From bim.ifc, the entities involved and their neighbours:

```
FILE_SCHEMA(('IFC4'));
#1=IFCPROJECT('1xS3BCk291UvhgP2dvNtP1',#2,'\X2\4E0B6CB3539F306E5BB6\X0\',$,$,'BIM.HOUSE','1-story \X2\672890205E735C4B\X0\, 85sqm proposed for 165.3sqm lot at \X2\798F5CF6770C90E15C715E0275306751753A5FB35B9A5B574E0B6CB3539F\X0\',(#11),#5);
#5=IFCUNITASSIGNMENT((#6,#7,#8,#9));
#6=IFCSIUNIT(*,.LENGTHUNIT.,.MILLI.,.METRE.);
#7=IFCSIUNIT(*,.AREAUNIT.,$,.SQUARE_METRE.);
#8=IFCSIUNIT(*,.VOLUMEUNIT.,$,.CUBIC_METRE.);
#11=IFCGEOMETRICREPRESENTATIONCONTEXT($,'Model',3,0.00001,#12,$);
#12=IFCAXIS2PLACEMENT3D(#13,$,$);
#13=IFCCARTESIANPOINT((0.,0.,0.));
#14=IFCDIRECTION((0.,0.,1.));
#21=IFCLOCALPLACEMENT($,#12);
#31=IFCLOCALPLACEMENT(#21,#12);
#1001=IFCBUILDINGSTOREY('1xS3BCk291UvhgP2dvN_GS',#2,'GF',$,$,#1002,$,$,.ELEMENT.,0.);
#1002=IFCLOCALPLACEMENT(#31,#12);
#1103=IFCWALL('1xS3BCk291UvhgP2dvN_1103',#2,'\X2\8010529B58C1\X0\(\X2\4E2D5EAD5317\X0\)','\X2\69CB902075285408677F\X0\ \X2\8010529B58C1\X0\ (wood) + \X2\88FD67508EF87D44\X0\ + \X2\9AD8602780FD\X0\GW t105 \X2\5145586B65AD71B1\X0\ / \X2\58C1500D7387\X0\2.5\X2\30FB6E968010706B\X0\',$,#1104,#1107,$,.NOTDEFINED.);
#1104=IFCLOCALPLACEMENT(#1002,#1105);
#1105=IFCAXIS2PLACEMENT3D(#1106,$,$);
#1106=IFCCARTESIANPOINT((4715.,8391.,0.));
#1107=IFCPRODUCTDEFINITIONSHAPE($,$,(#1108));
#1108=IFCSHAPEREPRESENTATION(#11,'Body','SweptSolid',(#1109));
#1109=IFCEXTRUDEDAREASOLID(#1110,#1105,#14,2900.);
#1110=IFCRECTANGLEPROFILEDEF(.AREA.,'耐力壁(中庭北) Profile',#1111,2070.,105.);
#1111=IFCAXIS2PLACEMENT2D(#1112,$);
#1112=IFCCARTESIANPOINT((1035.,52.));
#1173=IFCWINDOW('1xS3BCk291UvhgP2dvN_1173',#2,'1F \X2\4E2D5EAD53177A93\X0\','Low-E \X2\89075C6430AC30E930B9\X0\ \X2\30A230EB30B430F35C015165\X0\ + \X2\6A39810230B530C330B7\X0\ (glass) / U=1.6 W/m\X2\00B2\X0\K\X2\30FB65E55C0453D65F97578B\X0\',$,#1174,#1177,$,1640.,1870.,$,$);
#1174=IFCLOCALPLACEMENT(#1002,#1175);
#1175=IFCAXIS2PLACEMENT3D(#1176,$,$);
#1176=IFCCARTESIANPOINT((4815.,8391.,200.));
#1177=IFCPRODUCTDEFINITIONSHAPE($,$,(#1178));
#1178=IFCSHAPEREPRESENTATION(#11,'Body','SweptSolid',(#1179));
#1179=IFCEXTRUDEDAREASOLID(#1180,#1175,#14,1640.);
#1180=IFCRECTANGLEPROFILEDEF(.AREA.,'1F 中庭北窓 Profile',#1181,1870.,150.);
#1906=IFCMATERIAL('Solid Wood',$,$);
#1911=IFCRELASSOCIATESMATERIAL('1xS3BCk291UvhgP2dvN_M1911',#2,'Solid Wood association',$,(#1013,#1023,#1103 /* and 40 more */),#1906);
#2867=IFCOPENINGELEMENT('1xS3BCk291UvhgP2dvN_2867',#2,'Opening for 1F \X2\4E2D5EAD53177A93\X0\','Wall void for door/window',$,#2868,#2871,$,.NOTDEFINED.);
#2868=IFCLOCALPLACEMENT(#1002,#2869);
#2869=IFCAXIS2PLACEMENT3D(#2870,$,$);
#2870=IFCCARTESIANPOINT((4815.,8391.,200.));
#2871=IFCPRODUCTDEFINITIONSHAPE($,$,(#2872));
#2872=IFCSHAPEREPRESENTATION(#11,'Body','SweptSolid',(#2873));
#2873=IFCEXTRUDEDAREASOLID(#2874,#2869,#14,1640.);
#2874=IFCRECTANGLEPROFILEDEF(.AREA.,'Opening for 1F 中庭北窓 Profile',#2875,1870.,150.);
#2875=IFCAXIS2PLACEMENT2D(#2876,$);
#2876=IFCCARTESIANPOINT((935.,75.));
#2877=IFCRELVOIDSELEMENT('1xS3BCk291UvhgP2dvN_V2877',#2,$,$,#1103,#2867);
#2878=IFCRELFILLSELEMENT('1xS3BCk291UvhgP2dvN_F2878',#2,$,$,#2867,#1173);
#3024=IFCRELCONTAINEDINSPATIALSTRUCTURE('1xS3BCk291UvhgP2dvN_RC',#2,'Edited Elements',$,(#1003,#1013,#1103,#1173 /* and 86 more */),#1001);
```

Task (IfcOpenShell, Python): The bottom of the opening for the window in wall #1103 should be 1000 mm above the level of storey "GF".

```python
import numpy as np
import ifcopenshell
import ifcopenshell.api.geometry
import ifcopenshell.geom
import ifcopenshell.util.element
import ifcopenshell.util.placement
import ifcopenshell.util.shape
import ifcopenshell.util.unit

model = ifcopenshell.open("bim.ifc")
unit_scale = ifcopenshell.util.unit.calculate_unit_scale(model)

window = model.by_guid("1xS3BCk291UvhgP2dvN_1173")
opening = window.FillsVoids[0].RelatingOpeningElement
storey = ifcopenshell.util.element.get_container(window, ifc_class="IfcBuildingStorey")
level = ifcopenshell.util.placement.get_local_placement(storey.ObjectPlacement)[2, 3]

# The opening's origin need not be at the sill, so measure its lowest point.
shape = ifcopenshell.geom.create_shape(ifcopenshell.geom.settings(), opening)
bottom = ifcopenshell.util.shape.get_shape_bottom_elevation(shape, shape.geometry) / unit_scale
dz = level + 1000.0 - bottom

shift = np.array([0.0, 0.0, dz])
# The window is not placed relative to its opening, so move both.
for product in (opening, window):
    matrix = ifcopenshell.util.placement.get_local_placement(product.ObjectPlacement)
    matrix[:3, 3] += shift
    ifcopenshell.api.geometry.edit_object_placement(model, product=product, matrix=matrix, is_si=False)

print(f"moved by {dz * unit_scale:+.3f} m")

model.write("bim-out.ifc")
```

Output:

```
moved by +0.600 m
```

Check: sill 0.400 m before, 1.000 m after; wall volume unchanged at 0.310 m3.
